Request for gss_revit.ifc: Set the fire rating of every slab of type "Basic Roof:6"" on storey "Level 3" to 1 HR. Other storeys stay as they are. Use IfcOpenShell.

First a look at what the model holds.

```python
import ifcopenshell
import ifcopenshell.util.element

model = ifcopenshell.open("gss_revit.ifc")
print(model.schema)
storey = next(s for s in model.by_type("IfcBuildingStorey") if s.Name == "Level 3")
slabs = [e for e in ifcopenshell.util.element.get_decomposition(storey) if e.is_a("IfcSlab")]
seen = {}
for e in slabs:
    element_type = ifcopenshell.util.element.get_type(e)
    key = (element_type.Name if element_type != e and element_type else None, ifcopenshell.util.element.get_pset(e, "Pset_SlabCommon", "FireRating"))
    seen[key] = seen.get(key, 0) + 1
for (name, value), count in sorted(seen.items(), key=str):
    print(count, "x", name, "|", value)
```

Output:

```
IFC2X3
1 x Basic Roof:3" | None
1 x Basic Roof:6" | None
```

```python
import ifcopenshell
import ifcopenshell.api.pset
import ifcopenshell.util.element

model = ifcopenshell.open("gss_revit.ifc")

storey = next(s for s in model.by_type("IfcBuildingStorey") if s.Name == "Level 3")
slabs = [e for e in ifcopenshell.util.element.get_decomposition(storey) if e.is_a("IfcSlab")]

count = 0
for e in slabs:
    element_type = ifcopenshell.util.element.get_type(e)
    if element_type in (None, e) or element_type.Name != 'Basic Roof:6"':
        continue
    # add_pset returns the element's existing set when there is one.
    pset = ifcopenshell.api.pset.add_pset(model, product=e, name="Pset_SlabCommon")
    ifcopenshell.api.pset.edit_pset(model, pset=pset, properties={"FireRating": "1 HR"})
    count += 1

print(count, "slabs updated")

model.write("gss_revit_edited.ifc")
```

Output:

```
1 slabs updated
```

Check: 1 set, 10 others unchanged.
